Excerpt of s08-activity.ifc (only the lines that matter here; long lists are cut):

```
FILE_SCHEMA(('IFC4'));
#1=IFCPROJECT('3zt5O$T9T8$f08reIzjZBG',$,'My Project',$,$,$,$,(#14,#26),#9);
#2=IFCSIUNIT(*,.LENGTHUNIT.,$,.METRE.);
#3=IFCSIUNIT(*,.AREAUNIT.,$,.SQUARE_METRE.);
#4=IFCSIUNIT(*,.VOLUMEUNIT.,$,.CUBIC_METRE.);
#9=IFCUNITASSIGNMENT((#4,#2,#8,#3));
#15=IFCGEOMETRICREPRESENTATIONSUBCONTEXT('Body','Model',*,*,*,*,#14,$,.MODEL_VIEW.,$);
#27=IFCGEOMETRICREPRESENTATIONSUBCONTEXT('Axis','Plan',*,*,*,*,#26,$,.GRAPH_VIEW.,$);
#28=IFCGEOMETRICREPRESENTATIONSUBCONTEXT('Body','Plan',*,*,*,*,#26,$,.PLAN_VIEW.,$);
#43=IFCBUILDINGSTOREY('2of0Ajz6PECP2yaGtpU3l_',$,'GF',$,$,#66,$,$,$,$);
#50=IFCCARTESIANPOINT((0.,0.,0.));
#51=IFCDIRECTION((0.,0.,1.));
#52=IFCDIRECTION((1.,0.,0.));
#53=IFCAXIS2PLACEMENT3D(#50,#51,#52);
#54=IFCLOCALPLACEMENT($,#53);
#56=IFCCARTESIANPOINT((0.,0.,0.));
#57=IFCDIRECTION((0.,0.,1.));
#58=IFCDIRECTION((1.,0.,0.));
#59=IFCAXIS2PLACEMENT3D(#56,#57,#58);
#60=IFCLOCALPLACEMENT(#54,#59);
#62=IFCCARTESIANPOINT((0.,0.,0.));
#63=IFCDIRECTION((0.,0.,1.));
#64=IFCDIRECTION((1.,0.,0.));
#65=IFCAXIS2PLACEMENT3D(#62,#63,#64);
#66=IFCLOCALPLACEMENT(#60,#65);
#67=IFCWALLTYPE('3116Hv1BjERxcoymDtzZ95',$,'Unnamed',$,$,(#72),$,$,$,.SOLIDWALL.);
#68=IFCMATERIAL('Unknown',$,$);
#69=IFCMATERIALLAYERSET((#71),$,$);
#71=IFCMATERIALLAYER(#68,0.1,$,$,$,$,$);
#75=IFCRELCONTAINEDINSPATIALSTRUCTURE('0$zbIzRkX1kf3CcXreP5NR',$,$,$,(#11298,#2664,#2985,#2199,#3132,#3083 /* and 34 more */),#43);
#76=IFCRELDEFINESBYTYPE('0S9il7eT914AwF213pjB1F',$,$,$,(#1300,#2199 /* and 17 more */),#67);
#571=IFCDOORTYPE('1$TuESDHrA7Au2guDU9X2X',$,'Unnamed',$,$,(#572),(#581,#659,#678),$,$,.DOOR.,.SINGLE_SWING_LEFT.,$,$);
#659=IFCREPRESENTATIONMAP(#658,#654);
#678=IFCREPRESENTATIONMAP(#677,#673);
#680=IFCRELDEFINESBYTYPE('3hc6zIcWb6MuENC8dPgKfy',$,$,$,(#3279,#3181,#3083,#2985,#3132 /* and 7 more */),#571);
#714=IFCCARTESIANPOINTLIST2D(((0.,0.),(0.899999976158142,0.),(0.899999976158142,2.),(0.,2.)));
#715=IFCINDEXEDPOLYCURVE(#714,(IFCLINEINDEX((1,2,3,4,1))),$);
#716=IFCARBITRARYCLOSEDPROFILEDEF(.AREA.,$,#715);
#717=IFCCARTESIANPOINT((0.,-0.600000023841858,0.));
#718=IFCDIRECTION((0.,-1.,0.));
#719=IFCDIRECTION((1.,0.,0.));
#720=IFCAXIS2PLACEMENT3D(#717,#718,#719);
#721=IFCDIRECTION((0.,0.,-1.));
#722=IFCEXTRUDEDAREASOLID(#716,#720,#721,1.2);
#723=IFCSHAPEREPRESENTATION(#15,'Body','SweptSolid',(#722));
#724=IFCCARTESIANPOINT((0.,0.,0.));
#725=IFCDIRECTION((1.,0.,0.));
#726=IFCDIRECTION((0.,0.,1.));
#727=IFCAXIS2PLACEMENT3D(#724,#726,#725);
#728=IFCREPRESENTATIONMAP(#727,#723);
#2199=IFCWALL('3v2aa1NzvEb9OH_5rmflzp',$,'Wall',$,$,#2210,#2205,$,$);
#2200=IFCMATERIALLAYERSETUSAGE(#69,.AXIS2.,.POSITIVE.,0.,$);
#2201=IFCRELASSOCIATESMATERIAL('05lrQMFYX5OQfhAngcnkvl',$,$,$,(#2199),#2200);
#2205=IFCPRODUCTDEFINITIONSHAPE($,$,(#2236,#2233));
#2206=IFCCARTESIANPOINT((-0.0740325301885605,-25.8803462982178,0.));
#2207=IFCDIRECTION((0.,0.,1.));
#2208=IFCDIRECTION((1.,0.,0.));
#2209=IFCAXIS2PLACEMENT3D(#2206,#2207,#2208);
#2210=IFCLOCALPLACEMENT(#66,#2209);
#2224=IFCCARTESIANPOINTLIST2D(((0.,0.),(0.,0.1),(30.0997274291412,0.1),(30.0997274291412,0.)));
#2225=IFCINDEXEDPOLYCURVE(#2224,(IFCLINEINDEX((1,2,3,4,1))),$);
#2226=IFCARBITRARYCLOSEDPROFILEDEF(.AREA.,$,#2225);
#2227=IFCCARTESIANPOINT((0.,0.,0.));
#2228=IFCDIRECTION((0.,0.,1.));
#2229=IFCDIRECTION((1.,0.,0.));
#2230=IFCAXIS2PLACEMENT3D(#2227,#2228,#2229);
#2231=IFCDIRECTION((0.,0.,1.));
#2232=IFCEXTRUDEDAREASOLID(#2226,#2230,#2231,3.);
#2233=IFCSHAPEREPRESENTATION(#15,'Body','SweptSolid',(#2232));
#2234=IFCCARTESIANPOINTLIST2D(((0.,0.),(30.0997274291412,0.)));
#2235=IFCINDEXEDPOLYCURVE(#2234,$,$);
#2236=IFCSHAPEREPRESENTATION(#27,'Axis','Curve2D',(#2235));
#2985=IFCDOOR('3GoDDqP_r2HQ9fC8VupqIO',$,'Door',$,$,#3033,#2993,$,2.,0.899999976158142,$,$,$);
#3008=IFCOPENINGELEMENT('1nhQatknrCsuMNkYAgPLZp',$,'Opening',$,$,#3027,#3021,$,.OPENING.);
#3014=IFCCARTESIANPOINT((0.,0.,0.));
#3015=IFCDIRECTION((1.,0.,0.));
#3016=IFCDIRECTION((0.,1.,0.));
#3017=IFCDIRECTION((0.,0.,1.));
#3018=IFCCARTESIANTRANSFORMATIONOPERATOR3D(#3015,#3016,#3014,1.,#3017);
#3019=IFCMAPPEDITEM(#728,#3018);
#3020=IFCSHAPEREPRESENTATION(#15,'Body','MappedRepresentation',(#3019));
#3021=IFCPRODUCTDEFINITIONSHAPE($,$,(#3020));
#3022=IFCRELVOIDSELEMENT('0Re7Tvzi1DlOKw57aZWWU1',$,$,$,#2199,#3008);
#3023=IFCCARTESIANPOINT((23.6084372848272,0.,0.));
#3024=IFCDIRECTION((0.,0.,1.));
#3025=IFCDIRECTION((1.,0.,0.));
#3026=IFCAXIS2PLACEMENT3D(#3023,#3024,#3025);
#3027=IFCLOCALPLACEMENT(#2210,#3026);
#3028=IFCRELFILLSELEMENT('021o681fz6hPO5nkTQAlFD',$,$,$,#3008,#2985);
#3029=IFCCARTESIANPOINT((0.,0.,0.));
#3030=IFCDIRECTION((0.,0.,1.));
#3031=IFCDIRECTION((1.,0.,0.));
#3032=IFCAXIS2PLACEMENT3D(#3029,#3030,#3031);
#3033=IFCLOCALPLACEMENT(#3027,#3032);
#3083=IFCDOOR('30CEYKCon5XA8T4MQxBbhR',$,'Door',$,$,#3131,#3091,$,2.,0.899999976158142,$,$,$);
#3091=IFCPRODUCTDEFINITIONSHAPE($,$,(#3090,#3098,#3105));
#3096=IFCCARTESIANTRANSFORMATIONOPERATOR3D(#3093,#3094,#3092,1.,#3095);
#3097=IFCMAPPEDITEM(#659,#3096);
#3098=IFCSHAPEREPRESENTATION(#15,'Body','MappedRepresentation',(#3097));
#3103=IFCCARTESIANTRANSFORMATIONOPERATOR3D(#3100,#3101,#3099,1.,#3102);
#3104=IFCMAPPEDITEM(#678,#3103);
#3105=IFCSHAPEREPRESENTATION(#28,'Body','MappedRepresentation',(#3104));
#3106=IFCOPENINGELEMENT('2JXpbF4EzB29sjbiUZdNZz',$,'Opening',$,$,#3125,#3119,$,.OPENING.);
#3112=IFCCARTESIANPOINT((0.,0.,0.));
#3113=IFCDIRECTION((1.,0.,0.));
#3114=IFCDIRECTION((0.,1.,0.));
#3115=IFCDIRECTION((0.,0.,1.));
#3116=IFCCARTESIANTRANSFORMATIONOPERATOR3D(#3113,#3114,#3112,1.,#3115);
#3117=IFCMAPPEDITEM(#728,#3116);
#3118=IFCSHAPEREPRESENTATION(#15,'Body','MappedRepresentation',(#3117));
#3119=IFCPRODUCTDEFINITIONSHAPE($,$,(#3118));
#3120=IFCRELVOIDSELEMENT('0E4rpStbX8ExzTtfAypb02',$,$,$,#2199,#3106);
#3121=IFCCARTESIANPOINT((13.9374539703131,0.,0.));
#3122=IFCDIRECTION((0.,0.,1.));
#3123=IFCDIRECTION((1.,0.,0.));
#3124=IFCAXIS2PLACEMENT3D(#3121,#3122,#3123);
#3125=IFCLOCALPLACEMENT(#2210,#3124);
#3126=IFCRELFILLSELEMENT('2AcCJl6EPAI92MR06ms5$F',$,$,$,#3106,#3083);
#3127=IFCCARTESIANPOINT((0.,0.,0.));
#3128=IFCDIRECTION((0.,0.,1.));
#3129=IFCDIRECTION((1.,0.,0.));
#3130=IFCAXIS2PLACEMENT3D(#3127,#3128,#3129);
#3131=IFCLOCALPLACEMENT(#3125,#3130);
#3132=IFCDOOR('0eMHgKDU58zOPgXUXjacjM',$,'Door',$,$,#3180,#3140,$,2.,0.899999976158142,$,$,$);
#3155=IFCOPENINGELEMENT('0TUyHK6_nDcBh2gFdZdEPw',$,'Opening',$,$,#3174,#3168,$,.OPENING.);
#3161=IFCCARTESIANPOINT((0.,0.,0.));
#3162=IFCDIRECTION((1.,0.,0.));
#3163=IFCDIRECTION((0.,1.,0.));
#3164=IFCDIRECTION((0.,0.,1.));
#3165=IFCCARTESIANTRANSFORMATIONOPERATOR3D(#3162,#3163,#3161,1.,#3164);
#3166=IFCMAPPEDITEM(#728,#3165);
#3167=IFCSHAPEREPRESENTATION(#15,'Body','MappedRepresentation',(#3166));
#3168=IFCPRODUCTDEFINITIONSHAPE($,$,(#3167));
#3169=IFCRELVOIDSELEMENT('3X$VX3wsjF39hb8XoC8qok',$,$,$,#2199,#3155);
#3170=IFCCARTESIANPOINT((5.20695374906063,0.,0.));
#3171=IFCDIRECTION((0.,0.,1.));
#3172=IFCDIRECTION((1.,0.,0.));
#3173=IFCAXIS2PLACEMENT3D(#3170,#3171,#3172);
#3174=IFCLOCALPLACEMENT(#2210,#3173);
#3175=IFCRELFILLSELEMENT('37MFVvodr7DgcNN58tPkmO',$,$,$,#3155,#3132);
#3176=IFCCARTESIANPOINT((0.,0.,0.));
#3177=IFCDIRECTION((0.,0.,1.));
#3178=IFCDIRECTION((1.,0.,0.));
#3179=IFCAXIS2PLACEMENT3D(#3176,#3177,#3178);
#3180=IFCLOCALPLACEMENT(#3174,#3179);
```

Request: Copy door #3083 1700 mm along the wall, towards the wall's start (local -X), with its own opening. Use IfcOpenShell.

```python
import ifcopenshell
import ifcopenshell.api.feature
import ifcopenshell.api.geometry
import ifcopenshell.api.root
import ifcopenshell.geom
import ifcopenshell.util.element
import ifcopenshell.util.placement
import ifcopenshell.util.shape

model = ifcopenshell.open("s08-activity.ifc")
settings = ifcopenshell.geom.settings()


def volume(element):
    """Net volume in cubic metres, openings subtracted."""
    shape = ifcopenshell.geom.create_shape(settings, element)
    return ifcopenshell.util.shape.get_volume(shape.geometry)


door = model.by_guid("30CEYKCon5XA8T4MQxBbhR")
opening = door.FillsVoids[0].RelatingOpeningElement
wall = opening.VoidsElements[0].RelatingBuildingElement
before = volume(wall)
shift = ifcopenshell.util.placement.get_local_placement(wall.ObjectPlacement)[:3, 0] * -1.7

# copy_class copies the void relationship, type, container and properties, but no geometry.
new_opening = ifcopenshell.api.root.copy_class(model, product=opening)
new_opening.Representation = ifcopenshell.util.element.copy_deep(
    model, opening.Representation, exclude=["IfcGeometricRepresentationContext", "IfcRepresentationMap"]
)
new_door = ifcopenshell.api.root.copy_class(model, product=door)
new_door.Representation = ifcopenshell.util.element.copy_deep(
    model, door.Representation, exclude=["IfcGeometricRepresentationContext", "IfcRepresentationMap"]
)
ifcopenshell.api.feature.add_filling(model, opening=new_opening, element=new_door)

for old, new in ((opening, new_opening), (door, new_door)):
    matrix = ifcopenshell.util.placement.get_local_placement(old.ObjectPlacement)
    matrix[:3, 3] += shift
    ifcopenshell.api.geometry.edit_object_placement(model, product=new, matrix=matrix, is_si=False)

after = volume(wall)

print(f"wall volume {before:.3f} -> {after:.3f} m3")

model.write("s08-activity_rev.ifc")
```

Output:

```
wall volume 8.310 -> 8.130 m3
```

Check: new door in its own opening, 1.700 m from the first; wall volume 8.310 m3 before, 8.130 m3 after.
